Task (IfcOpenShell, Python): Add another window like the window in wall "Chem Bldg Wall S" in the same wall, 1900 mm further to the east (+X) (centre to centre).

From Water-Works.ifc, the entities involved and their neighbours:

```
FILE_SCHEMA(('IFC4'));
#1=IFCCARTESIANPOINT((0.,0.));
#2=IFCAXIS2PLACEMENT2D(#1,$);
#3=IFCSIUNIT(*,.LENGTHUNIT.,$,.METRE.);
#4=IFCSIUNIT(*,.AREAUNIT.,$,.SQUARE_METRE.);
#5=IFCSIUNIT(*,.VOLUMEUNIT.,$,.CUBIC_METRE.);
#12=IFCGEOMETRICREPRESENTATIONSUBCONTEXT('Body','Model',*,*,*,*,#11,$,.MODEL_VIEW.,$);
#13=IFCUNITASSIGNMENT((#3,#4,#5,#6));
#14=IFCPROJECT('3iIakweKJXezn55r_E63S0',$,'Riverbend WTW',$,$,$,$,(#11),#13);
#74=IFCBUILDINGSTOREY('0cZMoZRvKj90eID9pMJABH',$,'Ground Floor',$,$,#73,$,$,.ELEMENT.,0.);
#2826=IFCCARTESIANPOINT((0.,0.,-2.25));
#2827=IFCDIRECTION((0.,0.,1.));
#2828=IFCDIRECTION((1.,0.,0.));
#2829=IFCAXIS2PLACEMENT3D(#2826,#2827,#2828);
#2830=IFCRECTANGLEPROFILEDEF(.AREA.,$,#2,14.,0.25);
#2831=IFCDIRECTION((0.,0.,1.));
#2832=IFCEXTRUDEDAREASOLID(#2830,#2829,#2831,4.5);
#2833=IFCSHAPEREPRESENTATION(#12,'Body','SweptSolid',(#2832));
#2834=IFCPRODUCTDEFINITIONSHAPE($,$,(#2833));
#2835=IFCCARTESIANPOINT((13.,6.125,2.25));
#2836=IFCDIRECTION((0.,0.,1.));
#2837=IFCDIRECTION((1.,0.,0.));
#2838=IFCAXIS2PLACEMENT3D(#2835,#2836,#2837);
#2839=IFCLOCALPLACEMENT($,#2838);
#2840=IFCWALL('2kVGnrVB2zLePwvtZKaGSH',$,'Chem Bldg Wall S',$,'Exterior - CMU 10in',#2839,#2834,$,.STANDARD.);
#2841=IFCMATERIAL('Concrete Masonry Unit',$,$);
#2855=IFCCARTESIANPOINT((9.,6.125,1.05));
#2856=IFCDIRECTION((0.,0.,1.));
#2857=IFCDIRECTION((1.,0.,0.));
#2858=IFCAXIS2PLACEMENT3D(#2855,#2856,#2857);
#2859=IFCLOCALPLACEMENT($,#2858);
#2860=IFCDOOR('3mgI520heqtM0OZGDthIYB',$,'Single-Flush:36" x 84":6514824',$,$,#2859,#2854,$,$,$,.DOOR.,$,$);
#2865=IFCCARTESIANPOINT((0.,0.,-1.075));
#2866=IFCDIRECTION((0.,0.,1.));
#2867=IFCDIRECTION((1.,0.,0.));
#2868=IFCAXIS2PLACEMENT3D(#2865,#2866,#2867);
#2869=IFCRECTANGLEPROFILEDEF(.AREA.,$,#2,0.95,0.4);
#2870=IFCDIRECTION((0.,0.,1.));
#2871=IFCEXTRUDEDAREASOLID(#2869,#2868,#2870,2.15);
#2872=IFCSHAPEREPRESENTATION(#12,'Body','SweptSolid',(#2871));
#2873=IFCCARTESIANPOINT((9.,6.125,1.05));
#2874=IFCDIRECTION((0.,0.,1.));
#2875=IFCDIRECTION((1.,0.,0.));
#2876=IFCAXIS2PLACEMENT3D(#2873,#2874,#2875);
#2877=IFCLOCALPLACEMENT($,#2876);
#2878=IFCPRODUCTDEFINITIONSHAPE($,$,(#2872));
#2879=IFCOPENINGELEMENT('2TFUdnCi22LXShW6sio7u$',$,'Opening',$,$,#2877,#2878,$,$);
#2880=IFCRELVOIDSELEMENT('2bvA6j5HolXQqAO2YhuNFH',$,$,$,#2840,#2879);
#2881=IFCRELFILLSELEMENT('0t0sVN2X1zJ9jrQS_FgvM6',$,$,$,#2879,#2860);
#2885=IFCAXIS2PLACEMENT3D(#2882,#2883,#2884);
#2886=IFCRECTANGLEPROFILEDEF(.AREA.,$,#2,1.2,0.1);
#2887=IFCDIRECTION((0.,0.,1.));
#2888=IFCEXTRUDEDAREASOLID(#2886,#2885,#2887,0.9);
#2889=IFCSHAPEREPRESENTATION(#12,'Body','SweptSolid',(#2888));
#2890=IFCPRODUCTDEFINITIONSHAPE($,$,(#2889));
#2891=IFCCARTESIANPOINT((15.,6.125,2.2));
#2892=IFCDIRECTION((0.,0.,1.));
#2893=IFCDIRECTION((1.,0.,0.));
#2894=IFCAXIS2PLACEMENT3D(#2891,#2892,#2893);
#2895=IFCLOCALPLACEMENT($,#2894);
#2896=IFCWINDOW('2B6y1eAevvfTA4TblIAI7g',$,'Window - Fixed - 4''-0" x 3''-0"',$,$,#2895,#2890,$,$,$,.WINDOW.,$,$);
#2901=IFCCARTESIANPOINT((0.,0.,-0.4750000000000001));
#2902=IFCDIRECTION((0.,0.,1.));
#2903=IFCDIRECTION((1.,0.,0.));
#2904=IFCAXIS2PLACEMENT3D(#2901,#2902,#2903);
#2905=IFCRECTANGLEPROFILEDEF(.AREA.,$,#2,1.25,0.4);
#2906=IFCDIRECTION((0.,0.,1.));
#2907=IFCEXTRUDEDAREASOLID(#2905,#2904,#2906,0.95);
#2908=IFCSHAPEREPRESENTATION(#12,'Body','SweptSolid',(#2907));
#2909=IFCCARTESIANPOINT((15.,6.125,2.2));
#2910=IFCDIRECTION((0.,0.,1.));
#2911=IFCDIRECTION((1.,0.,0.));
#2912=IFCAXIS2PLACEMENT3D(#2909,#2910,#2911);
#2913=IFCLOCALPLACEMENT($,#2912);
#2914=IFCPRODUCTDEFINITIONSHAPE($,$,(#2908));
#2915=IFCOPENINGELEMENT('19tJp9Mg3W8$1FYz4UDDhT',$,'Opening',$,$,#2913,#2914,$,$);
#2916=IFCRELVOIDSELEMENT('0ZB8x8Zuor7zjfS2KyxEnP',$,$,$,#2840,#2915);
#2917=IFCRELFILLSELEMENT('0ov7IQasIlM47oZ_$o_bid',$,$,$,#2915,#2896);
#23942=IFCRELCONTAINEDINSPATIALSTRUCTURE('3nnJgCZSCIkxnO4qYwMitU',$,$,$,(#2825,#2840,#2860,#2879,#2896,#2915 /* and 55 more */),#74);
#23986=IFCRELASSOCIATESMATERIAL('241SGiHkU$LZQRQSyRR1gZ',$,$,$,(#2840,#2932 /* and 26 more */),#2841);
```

```python
import ifcopenshell
import ifcopenshell.api.feature
import ifcopenshell.api.geometry
import ifcopenshell.api.root
import ifcopenshell.geom
import ifcopenshell.util.element
import ifcopenshell.util.placement
import ifcopenshell.util.shape
import ifcopenshell.util.unit

model = ifcopenshell.open("Water-Works.ifc")
unit_scale = ifcopenshell.util.unit.calculate_unit_scale(model)
settings = ifcopenshell.geom.settings()


def volume(element):
    """Net volume in cubic metres, openings subtracted."""
    shape = ifcopenshell.geom.create_shape(settings, element)
    return ifcopenshell.util.shape.get_volume(shape.geometry)


window = model.by_guid("2B6y1eAevvfTA4TblIAI7g")
opening = window.FillsVoids[0].RelatingOpeningElement
wall = opening.VoidsElements[0].RelatingBuildingElement
before = volume(wall)
shift = ifcopenshell.util.placement.get_local_placement(wall.ObjectPlacement)[:3, 0] * 1.9 / unit_scale

# copy_class copies the void relationship, type, container and properties, but no geometry.
new_opening = ifcopenshell.api.root.copy_class(model, product=opening)
new_opening.Representation = ifcopenshell.util.element.copy_deep(
    model, opening.Representation, exclude=["IfcGeometricRepresentationContext", "IfcRepresentationMap"]
)
new_window = ifcopenshell.api.root.copy_class(model, product=window)
new_window.Representation = ifcopenshell.util.element.copy_deep(
    model, window.Representation, exclude=["IfcGeometricRepresentationContext", "IfcRepresentationMap"]
)
ifcopenshell.api.feature.add_filling(model, opening=new_opening, element=new_window)

for old, new in ((opening, new_opening), (window, new_window)):
    matrix = ifcopenshell.util.placement.get_local_placement(old.ObjectPlacement)
    matrix[:3, 3] += shift
    ifcopenshell.api.geometry.edit_object_placement(model, product=new, matrix=matrix, is_si=False)

after = volume(wall)

print(f"wall volume {before:.3f} -> {after:.3f} m3")

model.write("Water-Works_edited.ifc")
```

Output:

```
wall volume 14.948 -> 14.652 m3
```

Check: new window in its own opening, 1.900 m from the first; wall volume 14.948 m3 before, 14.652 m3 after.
